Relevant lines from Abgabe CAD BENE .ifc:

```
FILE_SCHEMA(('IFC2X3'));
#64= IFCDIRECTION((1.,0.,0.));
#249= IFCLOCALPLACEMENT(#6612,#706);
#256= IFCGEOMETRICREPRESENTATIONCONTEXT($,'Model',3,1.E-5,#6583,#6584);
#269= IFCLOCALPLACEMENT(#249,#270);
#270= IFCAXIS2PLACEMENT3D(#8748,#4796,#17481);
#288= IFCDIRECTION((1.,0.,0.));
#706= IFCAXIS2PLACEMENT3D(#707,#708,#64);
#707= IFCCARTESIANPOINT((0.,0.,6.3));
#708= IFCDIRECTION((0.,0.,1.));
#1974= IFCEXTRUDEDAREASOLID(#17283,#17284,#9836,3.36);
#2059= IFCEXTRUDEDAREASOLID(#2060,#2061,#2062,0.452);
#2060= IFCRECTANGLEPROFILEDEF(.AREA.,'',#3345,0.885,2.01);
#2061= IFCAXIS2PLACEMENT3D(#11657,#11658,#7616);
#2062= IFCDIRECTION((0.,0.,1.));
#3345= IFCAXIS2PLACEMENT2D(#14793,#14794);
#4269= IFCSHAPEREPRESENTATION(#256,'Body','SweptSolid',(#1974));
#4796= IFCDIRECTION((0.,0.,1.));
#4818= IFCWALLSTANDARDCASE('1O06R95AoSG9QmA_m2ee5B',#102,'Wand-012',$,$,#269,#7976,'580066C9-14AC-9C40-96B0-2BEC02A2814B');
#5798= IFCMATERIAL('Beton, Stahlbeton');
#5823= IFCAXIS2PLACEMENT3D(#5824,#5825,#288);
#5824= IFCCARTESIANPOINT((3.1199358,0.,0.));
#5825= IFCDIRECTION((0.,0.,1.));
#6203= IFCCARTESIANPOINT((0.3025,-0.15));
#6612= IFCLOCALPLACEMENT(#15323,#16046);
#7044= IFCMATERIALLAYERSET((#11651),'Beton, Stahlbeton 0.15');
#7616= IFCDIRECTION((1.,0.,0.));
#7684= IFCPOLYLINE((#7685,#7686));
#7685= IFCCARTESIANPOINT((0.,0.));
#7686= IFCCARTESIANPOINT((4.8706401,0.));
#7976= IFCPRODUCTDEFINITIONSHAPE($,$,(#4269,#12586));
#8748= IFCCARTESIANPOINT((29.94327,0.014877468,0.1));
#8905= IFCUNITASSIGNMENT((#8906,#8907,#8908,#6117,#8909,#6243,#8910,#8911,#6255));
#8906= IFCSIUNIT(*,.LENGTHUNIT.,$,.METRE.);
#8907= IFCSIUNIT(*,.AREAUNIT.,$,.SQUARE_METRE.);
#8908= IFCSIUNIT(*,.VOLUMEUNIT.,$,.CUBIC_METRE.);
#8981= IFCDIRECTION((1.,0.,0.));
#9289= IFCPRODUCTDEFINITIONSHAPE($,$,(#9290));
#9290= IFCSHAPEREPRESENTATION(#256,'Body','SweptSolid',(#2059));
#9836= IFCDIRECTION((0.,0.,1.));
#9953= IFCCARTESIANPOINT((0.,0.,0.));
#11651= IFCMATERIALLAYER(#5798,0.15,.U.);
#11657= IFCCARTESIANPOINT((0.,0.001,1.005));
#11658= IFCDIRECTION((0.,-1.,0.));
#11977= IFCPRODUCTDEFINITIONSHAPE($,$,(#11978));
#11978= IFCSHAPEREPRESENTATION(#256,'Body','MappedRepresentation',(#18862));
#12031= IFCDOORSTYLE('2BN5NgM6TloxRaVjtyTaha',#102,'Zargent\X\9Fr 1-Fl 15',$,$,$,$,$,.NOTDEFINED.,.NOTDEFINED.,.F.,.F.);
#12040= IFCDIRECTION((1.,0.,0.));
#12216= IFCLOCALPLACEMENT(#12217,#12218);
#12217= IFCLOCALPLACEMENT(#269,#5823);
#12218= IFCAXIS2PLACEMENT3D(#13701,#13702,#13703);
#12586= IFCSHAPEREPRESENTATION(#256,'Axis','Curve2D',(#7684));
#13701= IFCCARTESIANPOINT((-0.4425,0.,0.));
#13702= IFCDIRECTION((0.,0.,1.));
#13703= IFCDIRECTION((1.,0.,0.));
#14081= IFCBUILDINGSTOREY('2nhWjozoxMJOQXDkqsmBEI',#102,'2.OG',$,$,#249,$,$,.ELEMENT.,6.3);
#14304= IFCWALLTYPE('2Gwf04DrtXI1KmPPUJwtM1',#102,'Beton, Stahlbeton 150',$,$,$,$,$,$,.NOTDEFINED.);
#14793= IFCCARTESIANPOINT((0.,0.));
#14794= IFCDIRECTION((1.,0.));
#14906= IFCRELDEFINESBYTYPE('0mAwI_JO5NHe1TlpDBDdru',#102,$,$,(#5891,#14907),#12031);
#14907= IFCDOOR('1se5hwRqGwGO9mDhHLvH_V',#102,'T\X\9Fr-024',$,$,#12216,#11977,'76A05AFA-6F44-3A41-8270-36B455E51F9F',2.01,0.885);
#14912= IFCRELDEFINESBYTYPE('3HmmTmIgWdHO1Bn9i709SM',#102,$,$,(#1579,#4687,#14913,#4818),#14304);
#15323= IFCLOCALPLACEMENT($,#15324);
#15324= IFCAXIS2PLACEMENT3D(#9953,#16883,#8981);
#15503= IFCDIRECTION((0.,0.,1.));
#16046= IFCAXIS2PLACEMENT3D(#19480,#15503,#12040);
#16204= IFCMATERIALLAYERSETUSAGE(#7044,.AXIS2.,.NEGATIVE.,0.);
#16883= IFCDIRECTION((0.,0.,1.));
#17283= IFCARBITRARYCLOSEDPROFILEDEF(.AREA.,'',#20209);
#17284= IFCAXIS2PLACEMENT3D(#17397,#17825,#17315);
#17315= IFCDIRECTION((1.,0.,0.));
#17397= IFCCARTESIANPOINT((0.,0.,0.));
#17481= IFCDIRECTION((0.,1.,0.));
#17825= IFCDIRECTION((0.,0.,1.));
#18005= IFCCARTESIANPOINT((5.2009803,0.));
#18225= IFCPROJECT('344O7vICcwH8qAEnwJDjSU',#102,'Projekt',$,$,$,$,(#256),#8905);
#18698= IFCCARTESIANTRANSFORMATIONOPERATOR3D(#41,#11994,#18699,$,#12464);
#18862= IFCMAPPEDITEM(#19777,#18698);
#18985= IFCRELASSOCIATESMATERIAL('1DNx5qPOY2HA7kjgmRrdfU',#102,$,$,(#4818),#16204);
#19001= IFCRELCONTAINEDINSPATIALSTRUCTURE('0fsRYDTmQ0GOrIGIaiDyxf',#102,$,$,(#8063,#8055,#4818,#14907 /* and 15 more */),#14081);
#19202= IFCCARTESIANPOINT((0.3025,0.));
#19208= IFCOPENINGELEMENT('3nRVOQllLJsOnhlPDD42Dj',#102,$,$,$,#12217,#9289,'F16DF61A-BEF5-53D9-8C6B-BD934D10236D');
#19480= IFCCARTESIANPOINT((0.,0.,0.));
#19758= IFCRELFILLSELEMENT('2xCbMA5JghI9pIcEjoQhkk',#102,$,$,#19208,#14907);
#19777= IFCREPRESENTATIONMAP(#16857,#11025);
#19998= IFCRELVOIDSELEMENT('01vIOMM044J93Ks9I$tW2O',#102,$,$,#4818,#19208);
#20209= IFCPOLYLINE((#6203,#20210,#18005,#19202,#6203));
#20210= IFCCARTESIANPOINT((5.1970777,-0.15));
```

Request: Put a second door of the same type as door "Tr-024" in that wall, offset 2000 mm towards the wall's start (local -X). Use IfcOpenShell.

```python
import ifcopenshell
import ifcopenshell.api.feature
import ifcopenshell.api.geometry
import ifcopenshell.api.root
import ifcopenshell.geom
import ifcopenshell.util.element
import ifcopenshell.util.placement
import ifcopenshell.util.shape
import ifcopenshell.util.unit

model = ifcopenshell.open("Abgabe CAD BENE .ifc")
unit_scale = ifcopenshell.util.unit.calculate_unit_scale(model)
settings = ifcopenshell.geom.settings()


def volume(element):
    """Net volume in cubic metres, openings subtracted."""
    shape = ifcopenshell.geom.create_shape(settings, element)
    return ifcopenshell.util.shape.get_volume(shape.geometry)


def reuse_history(source, copy):
    """copy_class also copies each property set's owner history, people and application; keep the originals."""
    for rel in copy.IsDefinedBy:
        if rel.is_a("IfcRelDefinesByProperties") and (history := rel.RelatingPropertyDefinition.OwnerHistory):
            rel.RelatingPropertyDefinition.OwnerHistory = source.OwnerHistory
            ifcopenshell.util.element.remove_deep2(model, history)


door = model.by_guid("1se5hwRqGwGO9mDhHLvH_V")
opening = door.FillsVoids[0].RelatingOpeningElement
wall = opening.VoidsElements[0].RelatingBuildingElement
before = volume(wall)
shift = ifcopenshell.util.placement.get_local_placement(wall.ObjectPlacement)[:3, 0] * -2 / unit_scale

# copy_class copies the void relationship, type, container and properties, but no geometry.
new_opening = ifcopenshell.api.root.copy_class(model, product=opening)
new_opening.Representation = ifcopenshell.util.element.copy_deep(
    model, opening.Representation, exclude=["IfcGeometricRepresentationContext", "IfcRepresentationMap"]
)
new_opening.Tag = None
new_door = ifcopenshell.api.root.copy_class(model, product=door)
new_door.Representation = ifcopenshell.util.element.copy_deep(
    model, door.Representation, exclude=["IfcGeometricRepresentationContext", "IfcRepresentationMap"]
)
new_door.Tag = None
reuse_history(door, new_door)
fills = ifcopenshell.api.feature.add_filling(model, opening=new_opening, element=new_door)
fills.OwnerHistory = new_door.OwnerHistory  # required in IFC2X3

for old, new in ((opening, new_opening), (door, new_door)):
    matrix = ifcopenshell.util.placement.get_local_placement(old.ObjectPlacement)
    matrix[:3, 3] += shift
    ifcopenshell.api.geometry.edit_object_placement(model, product=new, matrix=matrix, is_si=False)

after = volume(wall)

print(f"wall volume {before:.3f} -> {after:.3f} m3")

model.write("Abgabe CAD BENE _edited.ifc")
```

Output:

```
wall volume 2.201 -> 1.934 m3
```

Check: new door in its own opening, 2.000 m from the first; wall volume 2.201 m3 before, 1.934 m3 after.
